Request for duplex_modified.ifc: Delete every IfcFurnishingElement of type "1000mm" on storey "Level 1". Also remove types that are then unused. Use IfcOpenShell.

First a look at what the model holds.

```python
import ifcopenshell
import ifcopenshell.util.element

model = ifcopenshell.open("duplex_modified.ifc")
print(model.schema)
storey = next(s for s in model.by_type("IfcBuildingStorey") if s.Name == "Level 1")
furniture = [e for e in ifcopenshell.util.element.get_decomposition(storey) if e.is_a("IfcFurnishingElement")]
seen = {}
for e in furniture:
    element_type = ifcopenshell.util.element.get_type(e)
    name = element_type.Name if element_type not in (None, e) else None
    seen[name] = seen.get(name, 0) + 1
for name, count in sorted(seen.items(), key=str):
    print(count, "x", name)
```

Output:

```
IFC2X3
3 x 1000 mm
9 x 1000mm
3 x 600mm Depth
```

```python
import ifcopenshell
import ifcopenshell.api.root
import ifcopenshell.util.element

model = ifcopenshell.open("duplex_modified.ifc")

storey = next(s for s in model.by_type("IfcBuildingStorey") if s.Name == "Level 1")
furniture = [e for e in ifcopenshell.util.element.get_decomposition(storey) if e.is_a("IfcFurnishingElement")]
targets = [e for e in furniture if (t := ifcopenshell.util.element.get_type(e)) not in (None, e) and t.Name == "1000mm"]
types = {ifcopenshell.util.element.get_type(e) for e in targets} - {None, *targets}

for e in targets:
    ifcopenshell.api.root.remove_product(model, product=e)
print(len(targets), "removed")

unused = [t for t in types if not ifcopenshell.util.element.get_types(t)]
for t in unused:
    ifcopenshell.api.root.remove_product(model, product=t)
print(len(unused), "unused types removed")

model.write("duplex_modified_updated.ifc")
```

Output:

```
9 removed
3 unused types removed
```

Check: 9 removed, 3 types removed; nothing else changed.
